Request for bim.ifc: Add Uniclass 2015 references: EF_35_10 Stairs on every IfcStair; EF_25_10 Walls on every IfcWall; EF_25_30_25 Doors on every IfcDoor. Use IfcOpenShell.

First a look at what the model holds.

```python
import ifcopenshell

model = ifcopenshell.open("bim.ifc")
print(model.schema)
print("classifications:", [c.Name for c in model.by_type("IfcClassification")])
for ifc_class in ("IfcDoor", "IfcRoof", "IfcStair", "IfcWall", "IfcWindow"):
    print(ifc_class, len(model.by_type(ifc_class)))
```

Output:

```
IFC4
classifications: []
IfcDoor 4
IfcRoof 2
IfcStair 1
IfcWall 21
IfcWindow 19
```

```python
import ifcopenshell
import ifcopenshell.api.classification

model = ifcopenshell.open("bim.ifc")

system = ifcopenshell.api.classification.add_classification(model, classification="Uniclass 2015")

codes = {
    "IfcStair": ("EF_35_10", "Stairs"),
    "IfcWall": ("EF_25_10", "Walls"),
    "IfcDoor": ("EF_25_30_25", "Doors"),
}
for ifc_class, (code, name) in codes.items():
    products = model.by_type(ifc_class)
    ifcopenshell.api.classification.add_reference(
        model, products=products, classification=system, identification=code, name=name
    )
    print(code, len(products))

model.write("bim-out.ifc")
```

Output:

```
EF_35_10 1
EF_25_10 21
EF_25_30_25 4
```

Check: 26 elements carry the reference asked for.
